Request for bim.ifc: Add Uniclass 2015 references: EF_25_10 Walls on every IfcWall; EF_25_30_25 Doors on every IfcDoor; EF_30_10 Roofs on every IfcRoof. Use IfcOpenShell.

First a look at what the model holds.

```python
import ifcopenshell

model = ifcopenshell.open("bim.ifc")
print(model.schema)
print("classifications:", [c.Name for c in model.by_type("IfcClassification")])
for ifc_class in ("IfcDoor", "IfcRoof", "IfcStair", "IfcWall", "IfcWindow"):
    print(ifc_class, len(model.by_type(ifc_class)))
```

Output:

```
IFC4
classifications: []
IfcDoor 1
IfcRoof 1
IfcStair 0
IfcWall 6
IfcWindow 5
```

```python
import ifcopenshell
import ifcopenshell.api.classification

model = ifcopenshell.open("bim.ifc")

system = ifcopenshell.api.classification.add_classification(model, classification="Uniclass 2015")

codes = {
    "IfcWall": ("EF_25_10", "Walls"),
    "IfcDoor": ("EF_25_30_25", "Doors"),
    "IfcRoof": ("EF_30_10", "Roofs"),
}
for ifc_class, (code, name) in codes.items():
    products = model.by_type(ifc_class)
    ifcopenshell.api.classification.add_reference(
        model, products=products, classification=system, identification=code, name=name
    )
    print(code, len(products))

model.write("bim-out.ifc")
```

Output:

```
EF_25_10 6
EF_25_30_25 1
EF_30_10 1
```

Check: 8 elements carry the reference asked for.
